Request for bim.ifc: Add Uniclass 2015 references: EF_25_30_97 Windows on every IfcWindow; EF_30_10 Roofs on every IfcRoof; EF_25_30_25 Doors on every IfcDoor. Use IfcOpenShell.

First a look at what the model holds.

```python
import ifcopenshell

model = ifcopenshell.open("bim.ifc")
print(model.schema)
print("classifications:", [c.Name for c in model.by_type("IfcClassification")])
for ifc_class in ("IfcDoor", "IfcRoof", "IfcStair", "IfcWall", "IfcWindow"):
    print(ifc_class, len(model.by_type(ifc_class)))
```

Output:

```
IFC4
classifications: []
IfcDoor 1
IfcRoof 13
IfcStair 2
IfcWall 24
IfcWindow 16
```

```python
import ifcopenshell
import ifcopenshell.api.classification

model = ifcopenshell.open("bim.ifc")

system = ifcopenshell.api.classification.add_classification(model, classification="Uniclass 2015")

codes = {
    "IfcWindow": ("EF_25_30_97", "Windows"),
    "IfcRoof": ("EF_30_10", "Roofs"),
    "IfcDoor": ("EF_25_30_25", "Doors"),
}
for ifc_class, (code, name) in codes.items():
    products = model.by_type(ifc_class)
    ifcopenshell.api.classification.add_reference(
        model, products=products, classification=system, identification=code, name=name
    )
    print(code, len(products))

model.write("bim_rev.ifc")
```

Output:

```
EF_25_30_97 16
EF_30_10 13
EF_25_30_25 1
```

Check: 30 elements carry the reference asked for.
